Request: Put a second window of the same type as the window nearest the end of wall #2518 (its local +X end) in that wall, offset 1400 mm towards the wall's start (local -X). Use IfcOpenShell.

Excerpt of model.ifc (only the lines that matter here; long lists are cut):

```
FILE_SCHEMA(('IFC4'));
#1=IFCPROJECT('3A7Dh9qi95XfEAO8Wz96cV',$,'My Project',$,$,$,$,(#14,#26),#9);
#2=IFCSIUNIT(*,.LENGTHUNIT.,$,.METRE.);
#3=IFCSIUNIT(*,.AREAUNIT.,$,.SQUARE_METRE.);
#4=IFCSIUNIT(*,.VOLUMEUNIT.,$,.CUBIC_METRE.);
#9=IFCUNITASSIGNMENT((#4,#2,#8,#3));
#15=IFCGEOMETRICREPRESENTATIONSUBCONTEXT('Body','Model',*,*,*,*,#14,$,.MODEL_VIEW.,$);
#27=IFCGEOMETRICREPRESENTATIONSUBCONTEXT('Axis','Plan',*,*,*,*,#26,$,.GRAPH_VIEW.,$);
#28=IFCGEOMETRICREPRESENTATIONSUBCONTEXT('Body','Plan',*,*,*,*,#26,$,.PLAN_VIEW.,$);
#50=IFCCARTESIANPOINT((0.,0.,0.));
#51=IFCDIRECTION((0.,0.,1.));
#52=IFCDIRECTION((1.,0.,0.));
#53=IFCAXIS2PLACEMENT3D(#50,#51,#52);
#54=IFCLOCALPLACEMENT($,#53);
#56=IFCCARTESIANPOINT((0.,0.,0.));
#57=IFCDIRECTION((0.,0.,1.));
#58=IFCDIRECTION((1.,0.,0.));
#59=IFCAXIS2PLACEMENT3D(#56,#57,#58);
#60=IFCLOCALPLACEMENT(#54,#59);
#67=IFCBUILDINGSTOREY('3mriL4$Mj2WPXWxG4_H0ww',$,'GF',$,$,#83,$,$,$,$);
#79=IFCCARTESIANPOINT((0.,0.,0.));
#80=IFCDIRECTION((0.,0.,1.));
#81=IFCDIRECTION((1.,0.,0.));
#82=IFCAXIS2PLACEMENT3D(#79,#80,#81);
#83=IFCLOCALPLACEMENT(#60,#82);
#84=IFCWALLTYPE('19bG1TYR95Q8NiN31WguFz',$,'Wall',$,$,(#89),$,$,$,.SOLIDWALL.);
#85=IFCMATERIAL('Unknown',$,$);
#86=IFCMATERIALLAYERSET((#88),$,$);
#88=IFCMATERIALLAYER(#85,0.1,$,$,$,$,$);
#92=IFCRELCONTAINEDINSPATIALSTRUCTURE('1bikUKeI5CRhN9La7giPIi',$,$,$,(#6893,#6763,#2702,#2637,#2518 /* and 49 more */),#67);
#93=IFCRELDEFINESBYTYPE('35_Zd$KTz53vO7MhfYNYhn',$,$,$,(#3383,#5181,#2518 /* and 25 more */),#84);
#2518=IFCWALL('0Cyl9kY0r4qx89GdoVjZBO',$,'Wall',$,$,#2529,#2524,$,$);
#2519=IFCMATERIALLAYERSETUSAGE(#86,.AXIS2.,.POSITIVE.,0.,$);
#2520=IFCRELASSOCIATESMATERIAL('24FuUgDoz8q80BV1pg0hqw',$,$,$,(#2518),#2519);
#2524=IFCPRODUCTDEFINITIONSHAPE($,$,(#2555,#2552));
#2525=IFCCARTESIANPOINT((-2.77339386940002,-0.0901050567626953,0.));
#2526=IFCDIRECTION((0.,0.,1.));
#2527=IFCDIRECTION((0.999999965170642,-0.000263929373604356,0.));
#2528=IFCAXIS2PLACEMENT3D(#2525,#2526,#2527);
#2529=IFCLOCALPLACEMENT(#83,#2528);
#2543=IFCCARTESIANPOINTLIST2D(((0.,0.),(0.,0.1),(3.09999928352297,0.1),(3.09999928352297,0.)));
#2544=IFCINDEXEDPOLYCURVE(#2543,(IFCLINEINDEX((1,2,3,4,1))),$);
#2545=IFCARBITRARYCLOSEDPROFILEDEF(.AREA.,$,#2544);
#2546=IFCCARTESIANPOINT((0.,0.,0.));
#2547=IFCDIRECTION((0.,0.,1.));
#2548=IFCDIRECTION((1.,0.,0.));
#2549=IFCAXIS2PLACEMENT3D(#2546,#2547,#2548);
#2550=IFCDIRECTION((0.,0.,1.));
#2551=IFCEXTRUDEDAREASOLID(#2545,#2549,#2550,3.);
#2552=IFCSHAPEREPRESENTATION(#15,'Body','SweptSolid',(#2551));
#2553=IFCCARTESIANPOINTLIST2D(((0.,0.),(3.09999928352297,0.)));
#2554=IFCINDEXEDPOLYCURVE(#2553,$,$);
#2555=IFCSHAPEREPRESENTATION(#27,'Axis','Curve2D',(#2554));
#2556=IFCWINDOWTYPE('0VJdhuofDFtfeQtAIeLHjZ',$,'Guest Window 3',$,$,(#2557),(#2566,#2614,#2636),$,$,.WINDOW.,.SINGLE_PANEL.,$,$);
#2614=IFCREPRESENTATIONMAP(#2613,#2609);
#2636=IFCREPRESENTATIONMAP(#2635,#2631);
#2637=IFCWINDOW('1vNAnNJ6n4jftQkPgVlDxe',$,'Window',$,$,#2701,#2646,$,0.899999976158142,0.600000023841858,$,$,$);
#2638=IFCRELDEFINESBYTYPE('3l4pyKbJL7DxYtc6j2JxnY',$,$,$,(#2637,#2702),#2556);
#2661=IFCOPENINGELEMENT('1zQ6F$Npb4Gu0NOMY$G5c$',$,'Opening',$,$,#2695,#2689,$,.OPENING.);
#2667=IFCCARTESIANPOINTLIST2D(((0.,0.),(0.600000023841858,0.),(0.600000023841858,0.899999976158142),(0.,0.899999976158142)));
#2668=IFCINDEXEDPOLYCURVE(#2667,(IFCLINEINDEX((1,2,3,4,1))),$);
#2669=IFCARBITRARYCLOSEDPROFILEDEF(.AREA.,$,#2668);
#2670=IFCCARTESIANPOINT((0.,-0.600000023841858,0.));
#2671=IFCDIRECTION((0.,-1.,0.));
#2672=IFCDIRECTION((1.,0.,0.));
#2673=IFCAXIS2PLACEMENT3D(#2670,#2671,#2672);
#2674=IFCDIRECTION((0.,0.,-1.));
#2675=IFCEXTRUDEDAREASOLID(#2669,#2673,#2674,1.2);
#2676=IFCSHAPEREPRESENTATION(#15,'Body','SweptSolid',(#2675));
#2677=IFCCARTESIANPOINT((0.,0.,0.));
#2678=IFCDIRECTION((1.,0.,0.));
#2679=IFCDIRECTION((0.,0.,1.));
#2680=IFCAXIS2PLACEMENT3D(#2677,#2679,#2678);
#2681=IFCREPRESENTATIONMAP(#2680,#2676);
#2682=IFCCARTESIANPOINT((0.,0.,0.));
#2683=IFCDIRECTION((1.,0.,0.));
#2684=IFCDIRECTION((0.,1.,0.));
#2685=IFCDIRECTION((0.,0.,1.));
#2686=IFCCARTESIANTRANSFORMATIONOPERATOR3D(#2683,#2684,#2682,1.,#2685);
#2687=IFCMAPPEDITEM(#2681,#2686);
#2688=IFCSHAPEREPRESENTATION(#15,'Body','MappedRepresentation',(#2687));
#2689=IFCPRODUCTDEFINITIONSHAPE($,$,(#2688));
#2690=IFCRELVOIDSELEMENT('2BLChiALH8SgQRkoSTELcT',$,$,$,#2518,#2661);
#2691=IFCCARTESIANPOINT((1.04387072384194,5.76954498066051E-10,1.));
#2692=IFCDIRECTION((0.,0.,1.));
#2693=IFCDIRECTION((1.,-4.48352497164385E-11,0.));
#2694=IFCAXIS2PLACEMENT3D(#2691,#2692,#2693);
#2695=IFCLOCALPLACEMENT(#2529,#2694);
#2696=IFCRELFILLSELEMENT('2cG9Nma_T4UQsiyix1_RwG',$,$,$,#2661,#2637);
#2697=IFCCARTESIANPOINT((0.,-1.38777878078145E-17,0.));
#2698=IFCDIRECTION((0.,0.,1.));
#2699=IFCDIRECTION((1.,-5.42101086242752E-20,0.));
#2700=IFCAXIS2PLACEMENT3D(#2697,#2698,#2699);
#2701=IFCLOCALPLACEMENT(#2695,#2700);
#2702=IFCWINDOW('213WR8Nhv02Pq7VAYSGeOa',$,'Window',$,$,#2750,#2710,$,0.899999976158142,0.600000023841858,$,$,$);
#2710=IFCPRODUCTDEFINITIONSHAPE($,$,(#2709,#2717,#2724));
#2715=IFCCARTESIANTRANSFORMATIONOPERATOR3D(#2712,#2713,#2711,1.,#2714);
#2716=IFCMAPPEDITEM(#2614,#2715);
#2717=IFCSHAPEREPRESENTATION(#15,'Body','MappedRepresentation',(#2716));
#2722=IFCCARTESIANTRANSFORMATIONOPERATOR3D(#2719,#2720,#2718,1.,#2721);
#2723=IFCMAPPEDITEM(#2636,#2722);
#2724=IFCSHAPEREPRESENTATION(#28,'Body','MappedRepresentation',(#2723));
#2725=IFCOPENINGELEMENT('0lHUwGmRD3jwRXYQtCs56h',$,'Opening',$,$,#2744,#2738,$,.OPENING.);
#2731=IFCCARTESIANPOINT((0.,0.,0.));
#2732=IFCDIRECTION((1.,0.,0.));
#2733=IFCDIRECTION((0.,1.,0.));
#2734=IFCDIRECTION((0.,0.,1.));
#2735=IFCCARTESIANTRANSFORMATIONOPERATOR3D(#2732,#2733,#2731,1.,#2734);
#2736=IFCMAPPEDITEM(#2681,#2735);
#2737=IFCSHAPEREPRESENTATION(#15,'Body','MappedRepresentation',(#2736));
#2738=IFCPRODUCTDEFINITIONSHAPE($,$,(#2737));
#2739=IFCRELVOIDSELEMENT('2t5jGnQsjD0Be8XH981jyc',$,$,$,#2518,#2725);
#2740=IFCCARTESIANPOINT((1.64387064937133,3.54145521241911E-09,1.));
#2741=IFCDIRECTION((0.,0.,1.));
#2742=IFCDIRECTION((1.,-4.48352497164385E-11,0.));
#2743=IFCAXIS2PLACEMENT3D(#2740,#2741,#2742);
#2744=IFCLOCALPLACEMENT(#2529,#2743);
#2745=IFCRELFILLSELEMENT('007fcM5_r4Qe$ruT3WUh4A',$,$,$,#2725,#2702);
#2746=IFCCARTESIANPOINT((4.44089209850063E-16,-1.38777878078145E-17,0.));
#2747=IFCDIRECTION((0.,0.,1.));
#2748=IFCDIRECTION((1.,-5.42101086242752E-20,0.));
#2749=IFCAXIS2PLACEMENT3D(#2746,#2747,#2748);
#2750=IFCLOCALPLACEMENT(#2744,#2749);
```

```python
import ifcopenshell
import ifcopenshell.api.feature
import ifcopenshell.api.geometry
import ifcopenshell.api.root
import ifcopenshell.geom
import ifcopenshell.util.element
import ifcopenshell.util.placement
import ifcopenshell.util.shape

model = ifcopenshell.open("model.ifc")
settings = ifcopenshell.geom.settings()


def volume(element):
    """Net volume in cubic metres, openings subtracted."""
    shape = ifcopenshell.geom.create_shape(settings, element)
    return ifcopenshell.util.shape.get_volume(shape.geometry)


window = model.by_id(2702)
opening = window.FillsVoids[0].RelatingOpeningElement
wall = opening.VoidsElements[0].RelatingBuildingElement
before = volume(wall)
shift = ifcopenshell.util.placement.get_local_placement(wall.ObjectPlacement)[:3, 0] * -1.4

# copy_class copies the void relationship, type, container and properties, but no geometry.
new_opening = ifcopenshell.api.root.copy_class(model, product=opening)
new_opening.Representation = ifcopenshell.util.element.copy_deep(
    model, opening.Representation, exclude=["IfcGeometricRepresentationContext", "IfcRepresentationMap"]
)
new_window = ifcopenshell.api.root.copy_class(model, product=window)
new_window.Representation = ifcopenshell.util.element.copy_deep(
    model, window.Representation, exclude=["IfcGeometricRepresentationContext", "IfcRepresentationMap"]
)
ifcopenshell.api.feature.add_filling(model, opening=new_opening, element=new_window)

for old, new in ((opening, new_opening), (window, new_window)):
    matrix = ifcopenshell.util.placement.get_local_placement(old.ObjectPlacement)
    matrix[:3, 3] += shift
    ifcopenshell.api.geometry.edit_object_placement(model, product=new, matrix=matrix, is_si=False)

after = volume(wall)

print(f"wall volume {before:.3f} -> {after:.3f} m3")

model.write("model_edited.ifc")
```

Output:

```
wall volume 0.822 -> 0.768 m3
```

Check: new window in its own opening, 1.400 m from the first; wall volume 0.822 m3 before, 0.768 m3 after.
